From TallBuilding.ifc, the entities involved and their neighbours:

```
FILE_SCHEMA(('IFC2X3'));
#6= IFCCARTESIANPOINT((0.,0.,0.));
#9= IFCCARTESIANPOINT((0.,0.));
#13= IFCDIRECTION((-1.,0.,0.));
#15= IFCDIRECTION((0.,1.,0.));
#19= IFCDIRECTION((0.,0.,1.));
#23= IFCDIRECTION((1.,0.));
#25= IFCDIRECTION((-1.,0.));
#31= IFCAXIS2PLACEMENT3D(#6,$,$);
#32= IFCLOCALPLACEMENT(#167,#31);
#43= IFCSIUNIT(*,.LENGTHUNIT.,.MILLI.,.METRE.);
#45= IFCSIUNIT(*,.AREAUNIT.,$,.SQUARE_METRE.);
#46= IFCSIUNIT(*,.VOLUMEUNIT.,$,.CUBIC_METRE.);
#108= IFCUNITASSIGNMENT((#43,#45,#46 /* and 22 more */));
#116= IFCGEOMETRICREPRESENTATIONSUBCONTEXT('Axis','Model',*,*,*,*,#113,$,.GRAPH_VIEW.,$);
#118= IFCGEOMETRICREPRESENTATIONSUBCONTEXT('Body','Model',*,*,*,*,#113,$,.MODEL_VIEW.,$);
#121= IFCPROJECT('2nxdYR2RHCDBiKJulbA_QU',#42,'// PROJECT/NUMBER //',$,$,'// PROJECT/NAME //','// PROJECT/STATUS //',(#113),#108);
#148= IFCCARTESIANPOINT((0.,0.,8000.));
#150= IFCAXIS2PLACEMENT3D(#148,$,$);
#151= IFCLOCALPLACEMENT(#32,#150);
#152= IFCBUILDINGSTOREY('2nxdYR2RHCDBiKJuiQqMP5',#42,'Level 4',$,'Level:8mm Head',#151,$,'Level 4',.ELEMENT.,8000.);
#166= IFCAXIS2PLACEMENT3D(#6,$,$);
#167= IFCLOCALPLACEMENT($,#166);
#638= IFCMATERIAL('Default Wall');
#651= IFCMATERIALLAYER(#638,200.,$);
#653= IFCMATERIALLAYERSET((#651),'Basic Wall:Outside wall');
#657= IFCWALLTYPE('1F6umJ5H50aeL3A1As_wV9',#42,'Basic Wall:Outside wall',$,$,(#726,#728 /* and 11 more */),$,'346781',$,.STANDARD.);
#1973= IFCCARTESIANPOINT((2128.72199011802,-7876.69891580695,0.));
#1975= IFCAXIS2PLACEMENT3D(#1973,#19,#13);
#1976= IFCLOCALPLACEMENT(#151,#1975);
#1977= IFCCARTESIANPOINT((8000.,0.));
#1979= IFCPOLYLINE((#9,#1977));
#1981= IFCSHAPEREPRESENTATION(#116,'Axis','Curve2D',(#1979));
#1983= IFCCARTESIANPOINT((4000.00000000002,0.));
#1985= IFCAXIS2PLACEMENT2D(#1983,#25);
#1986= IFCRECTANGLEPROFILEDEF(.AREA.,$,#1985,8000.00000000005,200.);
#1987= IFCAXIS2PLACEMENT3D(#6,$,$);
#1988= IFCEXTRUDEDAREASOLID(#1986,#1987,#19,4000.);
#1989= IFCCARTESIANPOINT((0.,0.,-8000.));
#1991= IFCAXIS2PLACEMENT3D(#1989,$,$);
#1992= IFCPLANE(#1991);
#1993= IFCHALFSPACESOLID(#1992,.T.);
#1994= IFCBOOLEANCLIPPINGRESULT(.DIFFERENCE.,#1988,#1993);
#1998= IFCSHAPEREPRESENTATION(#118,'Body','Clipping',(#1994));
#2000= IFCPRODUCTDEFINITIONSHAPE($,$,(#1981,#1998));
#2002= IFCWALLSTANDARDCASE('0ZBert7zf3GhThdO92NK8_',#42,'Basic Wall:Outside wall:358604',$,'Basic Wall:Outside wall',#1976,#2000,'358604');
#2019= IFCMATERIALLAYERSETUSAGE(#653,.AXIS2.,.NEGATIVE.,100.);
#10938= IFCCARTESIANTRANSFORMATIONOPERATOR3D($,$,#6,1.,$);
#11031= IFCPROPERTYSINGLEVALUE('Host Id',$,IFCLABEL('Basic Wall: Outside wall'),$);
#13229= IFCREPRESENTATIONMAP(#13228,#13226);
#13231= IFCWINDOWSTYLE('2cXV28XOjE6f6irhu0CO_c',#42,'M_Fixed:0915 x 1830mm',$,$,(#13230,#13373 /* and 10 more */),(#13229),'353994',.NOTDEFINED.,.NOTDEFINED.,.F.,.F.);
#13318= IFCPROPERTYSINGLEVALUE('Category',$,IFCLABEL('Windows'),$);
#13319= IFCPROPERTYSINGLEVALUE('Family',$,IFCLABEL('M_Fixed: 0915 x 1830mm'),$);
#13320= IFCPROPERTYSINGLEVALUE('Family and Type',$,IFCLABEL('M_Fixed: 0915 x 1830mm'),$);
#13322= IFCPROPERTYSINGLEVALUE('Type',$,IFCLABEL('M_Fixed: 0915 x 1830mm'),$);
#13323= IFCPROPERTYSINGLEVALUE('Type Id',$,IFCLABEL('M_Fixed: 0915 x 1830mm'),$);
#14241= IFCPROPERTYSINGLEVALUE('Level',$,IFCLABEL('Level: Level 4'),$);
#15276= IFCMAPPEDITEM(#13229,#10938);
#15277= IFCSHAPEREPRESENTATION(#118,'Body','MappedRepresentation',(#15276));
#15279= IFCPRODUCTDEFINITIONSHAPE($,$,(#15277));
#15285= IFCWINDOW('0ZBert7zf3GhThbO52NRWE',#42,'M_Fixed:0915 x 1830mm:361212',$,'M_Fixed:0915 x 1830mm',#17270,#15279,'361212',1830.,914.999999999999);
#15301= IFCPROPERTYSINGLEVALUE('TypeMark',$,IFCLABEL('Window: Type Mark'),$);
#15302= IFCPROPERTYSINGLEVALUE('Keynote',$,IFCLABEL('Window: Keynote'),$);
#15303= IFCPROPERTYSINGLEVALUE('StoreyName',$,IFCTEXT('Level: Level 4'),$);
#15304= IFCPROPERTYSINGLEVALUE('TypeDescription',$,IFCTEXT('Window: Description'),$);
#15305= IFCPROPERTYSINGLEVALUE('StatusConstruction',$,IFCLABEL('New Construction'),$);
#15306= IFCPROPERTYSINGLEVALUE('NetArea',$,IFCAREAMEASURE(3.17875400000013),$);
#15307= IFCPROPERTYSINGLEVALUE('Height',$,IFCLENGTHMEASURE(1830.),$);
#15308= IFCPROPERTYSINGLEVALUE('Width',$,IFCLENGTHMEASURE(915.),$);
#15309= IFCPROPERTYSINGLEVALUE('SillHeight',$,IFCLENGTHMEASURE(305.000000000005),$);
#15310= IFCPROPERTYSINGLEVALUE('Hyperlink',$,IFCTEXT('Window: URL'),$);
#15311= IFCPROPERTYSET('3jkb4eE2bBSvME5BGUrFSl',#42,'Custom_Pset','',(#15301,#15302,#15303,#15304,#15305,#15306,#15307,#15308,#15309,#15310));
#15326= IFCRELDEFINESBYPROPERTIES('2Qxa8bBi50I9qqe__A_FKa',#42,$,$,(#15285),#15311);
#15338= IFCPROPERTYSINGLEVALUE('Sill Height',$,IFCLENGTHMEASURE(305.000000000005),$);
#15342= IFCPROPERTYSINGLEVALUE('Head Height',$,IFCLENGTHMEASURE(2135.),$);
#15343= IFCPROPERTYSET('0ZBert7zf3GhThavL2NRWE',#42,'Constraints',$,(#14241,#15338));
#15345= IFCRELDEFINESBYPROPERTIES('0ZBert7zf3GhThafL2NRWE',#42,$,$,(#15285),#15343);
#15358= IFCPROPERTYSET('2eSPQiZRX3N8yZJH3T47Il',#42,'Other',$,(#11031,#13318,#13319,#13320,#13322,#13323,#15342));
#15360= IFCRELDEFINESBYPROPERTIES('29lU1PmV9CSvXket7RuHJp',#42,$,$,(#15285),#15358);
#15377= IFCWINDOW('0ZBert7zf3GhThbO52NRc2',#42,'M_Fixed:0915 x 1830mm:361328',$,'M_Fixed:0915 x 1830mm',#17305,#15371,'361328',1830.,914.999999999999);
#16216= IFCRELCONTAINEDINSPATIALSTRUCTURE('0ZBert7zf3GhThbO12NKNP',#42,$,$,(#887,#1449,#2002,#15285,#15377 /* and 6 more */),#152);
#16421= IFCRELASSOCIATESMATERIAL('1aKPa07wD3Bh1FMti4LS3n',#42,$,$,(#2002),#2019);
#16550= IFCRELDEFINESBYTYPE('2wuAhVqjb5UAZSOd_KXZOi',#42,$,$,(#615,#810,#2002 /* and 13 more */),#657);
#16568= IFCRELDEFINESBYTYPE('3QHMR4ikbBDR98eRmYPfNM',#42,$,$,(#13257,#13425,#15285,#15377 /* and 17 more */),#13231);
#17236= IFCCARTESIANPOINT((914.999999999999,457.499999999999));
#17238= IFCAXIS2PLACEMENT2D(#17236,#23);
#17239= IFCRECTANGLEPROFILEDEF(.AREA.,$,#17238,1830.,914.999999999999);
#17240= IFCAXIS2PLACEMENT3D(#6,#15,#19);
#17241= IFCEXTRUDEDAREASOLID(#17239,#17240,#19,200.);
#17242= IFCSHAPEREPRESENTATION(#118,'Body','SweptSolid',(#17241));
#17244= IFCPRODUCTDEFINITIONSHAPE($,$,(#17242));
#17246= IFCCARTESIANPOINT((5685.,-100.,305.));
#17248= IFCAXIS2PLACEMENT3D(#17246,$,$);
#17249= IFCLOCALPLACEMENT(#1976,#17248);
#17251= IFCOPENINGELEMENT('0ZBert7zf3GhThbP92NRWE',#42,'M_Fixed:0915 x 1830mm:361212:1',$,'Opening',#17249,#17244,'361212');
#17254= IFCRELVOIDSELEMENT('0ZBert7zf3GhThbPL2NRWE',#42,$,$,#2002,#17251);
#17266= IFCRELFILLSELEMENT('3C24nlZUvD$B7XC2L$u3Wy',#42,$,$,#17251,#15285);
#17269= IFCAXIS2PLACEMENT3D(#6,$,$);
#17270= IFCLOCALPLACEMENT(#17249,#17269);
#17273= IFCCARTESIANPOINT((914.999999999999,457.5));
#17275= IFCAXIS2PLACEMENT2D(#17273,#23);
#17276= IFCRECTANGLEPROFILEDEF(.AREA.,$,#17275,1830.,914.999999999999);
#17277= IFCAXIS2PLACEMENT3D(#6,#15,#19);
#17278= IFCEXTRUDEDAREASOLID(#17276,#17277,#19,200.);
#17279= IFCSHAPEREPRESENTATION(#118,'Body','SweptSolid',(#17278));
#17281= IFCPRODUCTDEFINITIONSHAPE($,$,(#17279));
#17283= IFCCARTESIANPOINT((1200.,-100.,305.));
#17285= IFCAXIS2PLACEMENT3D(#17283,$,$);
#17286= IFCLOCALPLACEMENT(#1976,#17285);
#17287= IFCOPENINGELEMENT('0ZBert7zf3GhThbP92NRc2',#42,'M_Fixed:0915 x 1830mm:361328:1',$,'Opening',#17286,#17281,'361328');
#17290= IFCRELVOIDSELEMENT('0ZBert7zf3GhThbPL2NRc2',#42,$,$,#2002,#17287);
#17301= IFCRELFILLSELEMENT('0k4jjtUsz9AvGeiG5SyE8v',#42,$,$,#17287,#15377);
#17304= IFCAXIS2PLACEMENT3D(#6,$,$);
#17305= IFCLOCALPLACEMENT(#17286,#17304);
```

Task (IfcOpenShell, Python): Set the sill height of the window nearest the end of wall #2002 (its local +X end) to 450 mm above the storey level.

```python
import numpy as np
import ifcopenshell
import ifcopenshell.api.geometry
import ifcopenshell.api.pset
import ifcopenshell.geom
import ifcopenshell.util.element
import ifcopenshell.util.placement
import ifcopenshell.util.shape
import ifcopenshell.util.unit

model = ifcopenshell.open("TallBuilding.ifc")
unit_scale = ifcopenshell.util.unit.calculate_unit_scale(model)

window = model.by_guid("0ZBert7zf3GhThbO52NRWE")
opening = window.FillsVoids[0].RelatingOpeningElement
storey = ifcopenshell.util.element.get_container(window, ifc_class="IfcBuildingStorey")
level = ifcopenshell.util.placement.get_local_placement(storey.ObjectPlacement)[2, 3]

# The opening's origin need not be at the sill, so measure its lowest point.
shape = ifcopenshell.geom.create_shape(ifcopenshell.geom.settings(), opening)
bottom = ifcopenshell.util.shape.get_shape_bottom_elevation(shape, shape.geometry) / unit_scale
dz = level + 450.0 - bottom

shift = np.array([0.0, 0.0, dz])
# The window is placed relative to its opening, so it follows when the opening moves.
matrix = ifcopenshell.util.placement.get_local_placement(opening.ObjectPlacement)
matrix[:3, 3] += shift
ifcopenshell.api.geometry.edit_object_placement(
    model, product=opening, matrix=matrix, is_si=False, should_transform_children=True
)

# Keep the stored heights in step.
pset = model.by_id(ifcopenshell.util.element.get_pset(window, "Custom_Pset", should_inherit=False)["id"])
ifcopenshell.api.pset.edit_pset(model, pset=pset, properties={
    "SillHeight": model.create_entity("IfcLengthMeasure", ifcopenshell.util.element.get_pset(window, "Constraints", "Sill Height") + dz),
})
pset = model.by_id(ifcopenshell.util.element.get_pset(window, "Constraints", should_inherit=False)["id"])
ifcopenshell.api.pset.edit_pset(model, pset=pset, properties={
    "Sill Height": model.create_entity("IfcLengthMeasure", ifcopenshell.util.element.get_pset(window, "Constraints", "Sill Height") + dz),
})
pset = model.by_id(ifcopenshell.util.element.get_pset(window, "Other", should_inherit=False)["id"])
ifcopenshell.api.pset.edit_pset(model, pset=pset, properties={
    "Head Height": model.create_entity("IfcLengthMeasure", ifcopenshell.util.element.get_pset(window, "Other", "Head Height") + dz),
})

print(f"moved by {dz * unit_scale:+.3f} m")

model.write("TallBuilding_rev.ifc")
```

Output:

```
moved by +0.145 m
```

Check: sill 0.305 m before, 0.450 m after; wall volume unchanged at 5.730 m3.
